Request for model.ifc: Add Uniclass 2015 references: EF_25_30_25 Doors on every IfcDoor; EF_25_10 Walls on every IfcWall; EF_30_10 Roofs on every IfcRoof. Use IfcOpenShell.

First a look at what the model holds.

```python
import ifcopenshell

model = ifcopenshell.open("model.ifc")
print(model.schema)
print("classifications:", [c.Name for c in model.by_type("IfcClassification")])
for ifc_class in ("IfcDoor", "IfcRoof", "IfcStair", "IfcWall", "IfcWindow"):
    print(ifc_class, len(model.by_type(ifc_class)))
```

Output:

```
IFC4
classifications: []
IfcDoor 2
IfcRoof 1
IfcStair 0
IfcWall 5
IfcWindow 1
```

```python
import ifcopenshell
import ifcopenshell.api.classification

model = ifcopenshell.open("model.ifc")

system = ifcopenshell.api.classification.add_classification(model, classification="Uniclass 2015")

codes = {
    "IfcDoor": ("EF_25_30_25", "Doors"),
    "IfcWall": ("EF_25_10", "Walls"),
    "IfcRoof": ("EF_30_10", "Roofs"),
}
for ifc_class, (code, name) in codes.items():
    products = model.by_type(ifc_class)
    ifcopenshell.api.classification.add_reference(
        model, products=products, classification=system, identification=code, name=name
    )
    print(code, len(products))

model.write("model_rev.ifc")
```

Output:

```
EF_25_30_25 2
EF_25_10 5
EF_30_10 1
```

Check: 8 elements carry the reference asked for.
